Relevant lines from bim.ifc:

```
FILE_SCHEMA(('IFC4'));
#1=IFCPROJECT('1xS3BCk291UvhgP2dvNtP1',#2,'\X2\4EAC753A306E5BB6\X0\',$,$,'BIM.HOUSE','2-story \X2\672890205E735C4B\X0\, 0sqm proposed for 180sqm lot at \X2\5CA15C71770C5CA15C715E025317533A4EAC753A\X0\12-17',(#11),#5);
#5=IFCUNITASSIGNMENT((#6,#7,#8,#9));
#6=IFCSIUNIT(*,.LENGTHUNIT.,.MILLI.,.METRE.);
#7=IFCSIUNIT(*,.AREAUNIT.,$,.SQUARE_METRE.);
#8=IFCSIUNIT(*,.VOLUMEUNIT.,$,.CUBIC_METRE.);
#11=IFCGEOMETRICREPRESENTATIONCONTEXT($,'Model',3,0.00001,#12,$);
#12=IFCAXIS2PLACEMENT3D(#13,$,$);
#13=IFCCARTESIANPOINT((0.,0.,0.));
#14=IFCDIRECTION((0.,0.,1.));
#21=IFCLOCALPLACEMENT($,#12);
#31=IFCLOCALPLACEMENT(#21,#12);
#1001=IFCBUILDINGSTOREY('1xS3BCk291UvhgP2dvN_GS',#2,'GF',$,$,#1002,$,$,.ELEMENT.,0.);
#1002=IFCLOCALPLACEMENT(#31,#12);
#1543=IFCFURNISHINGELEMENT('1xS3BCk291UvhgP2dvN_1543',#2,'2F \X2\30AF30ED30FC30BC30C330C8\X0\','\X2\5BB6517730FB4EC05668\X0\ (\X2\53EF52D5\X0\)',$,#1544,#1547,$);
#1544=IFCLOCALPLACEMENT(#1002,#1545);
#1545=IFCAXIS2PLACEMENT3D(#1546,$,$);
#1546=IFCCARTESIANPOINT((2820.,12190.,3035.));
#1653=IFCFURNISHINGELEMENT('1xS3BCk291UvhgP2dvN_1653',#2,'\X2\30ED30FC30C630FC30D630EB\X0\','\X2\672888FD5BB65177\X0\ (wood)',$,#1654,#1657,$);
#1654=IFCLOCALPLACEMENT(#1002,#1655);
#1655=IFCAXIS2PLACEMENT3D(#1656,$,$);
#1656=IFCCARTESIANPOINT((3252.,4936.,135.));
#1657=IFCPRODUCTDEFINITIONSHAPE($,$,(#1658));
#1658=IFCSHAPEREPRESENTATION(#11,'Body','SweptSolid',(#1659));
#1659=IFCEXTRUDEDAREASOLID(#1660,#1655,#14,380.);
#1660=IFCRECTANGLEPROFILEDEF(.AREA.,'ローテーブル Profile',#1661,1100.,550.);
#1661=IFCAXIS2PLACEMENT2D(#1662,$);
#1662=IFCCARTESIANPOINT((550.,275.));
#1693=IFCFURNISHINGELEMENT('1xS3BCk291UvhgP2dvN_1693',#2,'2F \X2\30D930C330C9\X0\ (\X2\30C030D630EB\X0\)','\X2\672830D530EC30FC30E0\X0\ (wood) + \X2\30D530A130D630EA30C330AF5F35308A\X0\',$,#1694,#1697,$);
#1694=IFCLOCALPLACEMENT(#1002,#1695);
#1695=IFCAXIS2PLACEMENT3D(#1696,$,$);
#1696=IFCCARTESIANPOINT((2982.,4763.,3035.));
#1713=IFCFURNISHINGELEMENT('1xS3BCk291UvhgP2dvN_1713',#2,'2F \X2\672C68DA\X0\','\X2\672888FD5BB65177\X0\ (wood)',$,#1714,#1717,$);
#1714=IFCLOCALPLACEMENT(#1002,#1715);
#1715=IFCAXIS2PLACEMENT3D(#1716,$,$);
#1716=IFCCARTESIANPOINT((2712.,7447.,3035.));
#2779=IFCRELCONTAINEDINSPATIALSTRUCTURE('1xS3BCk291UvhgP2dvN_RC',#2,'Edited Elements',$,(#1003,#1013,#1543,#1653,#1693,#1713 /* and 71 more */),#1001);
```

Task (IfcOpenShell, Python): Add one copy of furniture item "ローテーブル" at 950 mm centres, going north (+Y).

```python
import numpy as np
import ifcopenshell
import ifcopenshell.api.geometry
import ifcopenshell.api.root
import ifcopenshell.util.element
import ifcopenshell.util.placement
import ifcopenshell.util.unit

model = ifcopenshell.open("bim.ifc")
unit_scale = ifcopenshell.util.unit.calculate_unit_scale(model)


def reuse_history(source, copy):
    """copy_class also copies each property set's owner history, people and application; keep the originals."""
    for rel in copy.IsDefinedBy:
        if rel.is_a("IfcRelDefinesByProperties") and (history := rel.RelatingPropertyDefinition.OwnerHistory):
            rel.RelatingPropertyDefinition.OwnerHistory = source.OwnerHistory
            ifcopenshell.util.element.remove_deep2(model, history)


source = model.by_id(1653)
base = ifcopenshell.util.placement.get_local_placement(source.ObjectPlacement)
step = np.array([0.0, 1.0, 0.0]) * 0.95 / unit_scale

for i in range(1, 2):
    copy = ifcopenshell.api.root.copy_class(model, product=source)
    copy.Representation = ifcopenshell.util.element.copy_deep(
        model, source.Representation, exclude=["IfcGeometricRepresentationContext", "IfcRepresentationMap"]
    )
    reuse_history(source, copy)
    matrix = base.copy()
    matrix[:3, 3] += i * step
    print("added at", matrix[:3, 3].round(3) + 0.0)
    ifcopenshell.api.geometry.edit_object_placement(model, product=copy, matrix=matrix, is_si=False)

model.write("bim_v2.ifc")
```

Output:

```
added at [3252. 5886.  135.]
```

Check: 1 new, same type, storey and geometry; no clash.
